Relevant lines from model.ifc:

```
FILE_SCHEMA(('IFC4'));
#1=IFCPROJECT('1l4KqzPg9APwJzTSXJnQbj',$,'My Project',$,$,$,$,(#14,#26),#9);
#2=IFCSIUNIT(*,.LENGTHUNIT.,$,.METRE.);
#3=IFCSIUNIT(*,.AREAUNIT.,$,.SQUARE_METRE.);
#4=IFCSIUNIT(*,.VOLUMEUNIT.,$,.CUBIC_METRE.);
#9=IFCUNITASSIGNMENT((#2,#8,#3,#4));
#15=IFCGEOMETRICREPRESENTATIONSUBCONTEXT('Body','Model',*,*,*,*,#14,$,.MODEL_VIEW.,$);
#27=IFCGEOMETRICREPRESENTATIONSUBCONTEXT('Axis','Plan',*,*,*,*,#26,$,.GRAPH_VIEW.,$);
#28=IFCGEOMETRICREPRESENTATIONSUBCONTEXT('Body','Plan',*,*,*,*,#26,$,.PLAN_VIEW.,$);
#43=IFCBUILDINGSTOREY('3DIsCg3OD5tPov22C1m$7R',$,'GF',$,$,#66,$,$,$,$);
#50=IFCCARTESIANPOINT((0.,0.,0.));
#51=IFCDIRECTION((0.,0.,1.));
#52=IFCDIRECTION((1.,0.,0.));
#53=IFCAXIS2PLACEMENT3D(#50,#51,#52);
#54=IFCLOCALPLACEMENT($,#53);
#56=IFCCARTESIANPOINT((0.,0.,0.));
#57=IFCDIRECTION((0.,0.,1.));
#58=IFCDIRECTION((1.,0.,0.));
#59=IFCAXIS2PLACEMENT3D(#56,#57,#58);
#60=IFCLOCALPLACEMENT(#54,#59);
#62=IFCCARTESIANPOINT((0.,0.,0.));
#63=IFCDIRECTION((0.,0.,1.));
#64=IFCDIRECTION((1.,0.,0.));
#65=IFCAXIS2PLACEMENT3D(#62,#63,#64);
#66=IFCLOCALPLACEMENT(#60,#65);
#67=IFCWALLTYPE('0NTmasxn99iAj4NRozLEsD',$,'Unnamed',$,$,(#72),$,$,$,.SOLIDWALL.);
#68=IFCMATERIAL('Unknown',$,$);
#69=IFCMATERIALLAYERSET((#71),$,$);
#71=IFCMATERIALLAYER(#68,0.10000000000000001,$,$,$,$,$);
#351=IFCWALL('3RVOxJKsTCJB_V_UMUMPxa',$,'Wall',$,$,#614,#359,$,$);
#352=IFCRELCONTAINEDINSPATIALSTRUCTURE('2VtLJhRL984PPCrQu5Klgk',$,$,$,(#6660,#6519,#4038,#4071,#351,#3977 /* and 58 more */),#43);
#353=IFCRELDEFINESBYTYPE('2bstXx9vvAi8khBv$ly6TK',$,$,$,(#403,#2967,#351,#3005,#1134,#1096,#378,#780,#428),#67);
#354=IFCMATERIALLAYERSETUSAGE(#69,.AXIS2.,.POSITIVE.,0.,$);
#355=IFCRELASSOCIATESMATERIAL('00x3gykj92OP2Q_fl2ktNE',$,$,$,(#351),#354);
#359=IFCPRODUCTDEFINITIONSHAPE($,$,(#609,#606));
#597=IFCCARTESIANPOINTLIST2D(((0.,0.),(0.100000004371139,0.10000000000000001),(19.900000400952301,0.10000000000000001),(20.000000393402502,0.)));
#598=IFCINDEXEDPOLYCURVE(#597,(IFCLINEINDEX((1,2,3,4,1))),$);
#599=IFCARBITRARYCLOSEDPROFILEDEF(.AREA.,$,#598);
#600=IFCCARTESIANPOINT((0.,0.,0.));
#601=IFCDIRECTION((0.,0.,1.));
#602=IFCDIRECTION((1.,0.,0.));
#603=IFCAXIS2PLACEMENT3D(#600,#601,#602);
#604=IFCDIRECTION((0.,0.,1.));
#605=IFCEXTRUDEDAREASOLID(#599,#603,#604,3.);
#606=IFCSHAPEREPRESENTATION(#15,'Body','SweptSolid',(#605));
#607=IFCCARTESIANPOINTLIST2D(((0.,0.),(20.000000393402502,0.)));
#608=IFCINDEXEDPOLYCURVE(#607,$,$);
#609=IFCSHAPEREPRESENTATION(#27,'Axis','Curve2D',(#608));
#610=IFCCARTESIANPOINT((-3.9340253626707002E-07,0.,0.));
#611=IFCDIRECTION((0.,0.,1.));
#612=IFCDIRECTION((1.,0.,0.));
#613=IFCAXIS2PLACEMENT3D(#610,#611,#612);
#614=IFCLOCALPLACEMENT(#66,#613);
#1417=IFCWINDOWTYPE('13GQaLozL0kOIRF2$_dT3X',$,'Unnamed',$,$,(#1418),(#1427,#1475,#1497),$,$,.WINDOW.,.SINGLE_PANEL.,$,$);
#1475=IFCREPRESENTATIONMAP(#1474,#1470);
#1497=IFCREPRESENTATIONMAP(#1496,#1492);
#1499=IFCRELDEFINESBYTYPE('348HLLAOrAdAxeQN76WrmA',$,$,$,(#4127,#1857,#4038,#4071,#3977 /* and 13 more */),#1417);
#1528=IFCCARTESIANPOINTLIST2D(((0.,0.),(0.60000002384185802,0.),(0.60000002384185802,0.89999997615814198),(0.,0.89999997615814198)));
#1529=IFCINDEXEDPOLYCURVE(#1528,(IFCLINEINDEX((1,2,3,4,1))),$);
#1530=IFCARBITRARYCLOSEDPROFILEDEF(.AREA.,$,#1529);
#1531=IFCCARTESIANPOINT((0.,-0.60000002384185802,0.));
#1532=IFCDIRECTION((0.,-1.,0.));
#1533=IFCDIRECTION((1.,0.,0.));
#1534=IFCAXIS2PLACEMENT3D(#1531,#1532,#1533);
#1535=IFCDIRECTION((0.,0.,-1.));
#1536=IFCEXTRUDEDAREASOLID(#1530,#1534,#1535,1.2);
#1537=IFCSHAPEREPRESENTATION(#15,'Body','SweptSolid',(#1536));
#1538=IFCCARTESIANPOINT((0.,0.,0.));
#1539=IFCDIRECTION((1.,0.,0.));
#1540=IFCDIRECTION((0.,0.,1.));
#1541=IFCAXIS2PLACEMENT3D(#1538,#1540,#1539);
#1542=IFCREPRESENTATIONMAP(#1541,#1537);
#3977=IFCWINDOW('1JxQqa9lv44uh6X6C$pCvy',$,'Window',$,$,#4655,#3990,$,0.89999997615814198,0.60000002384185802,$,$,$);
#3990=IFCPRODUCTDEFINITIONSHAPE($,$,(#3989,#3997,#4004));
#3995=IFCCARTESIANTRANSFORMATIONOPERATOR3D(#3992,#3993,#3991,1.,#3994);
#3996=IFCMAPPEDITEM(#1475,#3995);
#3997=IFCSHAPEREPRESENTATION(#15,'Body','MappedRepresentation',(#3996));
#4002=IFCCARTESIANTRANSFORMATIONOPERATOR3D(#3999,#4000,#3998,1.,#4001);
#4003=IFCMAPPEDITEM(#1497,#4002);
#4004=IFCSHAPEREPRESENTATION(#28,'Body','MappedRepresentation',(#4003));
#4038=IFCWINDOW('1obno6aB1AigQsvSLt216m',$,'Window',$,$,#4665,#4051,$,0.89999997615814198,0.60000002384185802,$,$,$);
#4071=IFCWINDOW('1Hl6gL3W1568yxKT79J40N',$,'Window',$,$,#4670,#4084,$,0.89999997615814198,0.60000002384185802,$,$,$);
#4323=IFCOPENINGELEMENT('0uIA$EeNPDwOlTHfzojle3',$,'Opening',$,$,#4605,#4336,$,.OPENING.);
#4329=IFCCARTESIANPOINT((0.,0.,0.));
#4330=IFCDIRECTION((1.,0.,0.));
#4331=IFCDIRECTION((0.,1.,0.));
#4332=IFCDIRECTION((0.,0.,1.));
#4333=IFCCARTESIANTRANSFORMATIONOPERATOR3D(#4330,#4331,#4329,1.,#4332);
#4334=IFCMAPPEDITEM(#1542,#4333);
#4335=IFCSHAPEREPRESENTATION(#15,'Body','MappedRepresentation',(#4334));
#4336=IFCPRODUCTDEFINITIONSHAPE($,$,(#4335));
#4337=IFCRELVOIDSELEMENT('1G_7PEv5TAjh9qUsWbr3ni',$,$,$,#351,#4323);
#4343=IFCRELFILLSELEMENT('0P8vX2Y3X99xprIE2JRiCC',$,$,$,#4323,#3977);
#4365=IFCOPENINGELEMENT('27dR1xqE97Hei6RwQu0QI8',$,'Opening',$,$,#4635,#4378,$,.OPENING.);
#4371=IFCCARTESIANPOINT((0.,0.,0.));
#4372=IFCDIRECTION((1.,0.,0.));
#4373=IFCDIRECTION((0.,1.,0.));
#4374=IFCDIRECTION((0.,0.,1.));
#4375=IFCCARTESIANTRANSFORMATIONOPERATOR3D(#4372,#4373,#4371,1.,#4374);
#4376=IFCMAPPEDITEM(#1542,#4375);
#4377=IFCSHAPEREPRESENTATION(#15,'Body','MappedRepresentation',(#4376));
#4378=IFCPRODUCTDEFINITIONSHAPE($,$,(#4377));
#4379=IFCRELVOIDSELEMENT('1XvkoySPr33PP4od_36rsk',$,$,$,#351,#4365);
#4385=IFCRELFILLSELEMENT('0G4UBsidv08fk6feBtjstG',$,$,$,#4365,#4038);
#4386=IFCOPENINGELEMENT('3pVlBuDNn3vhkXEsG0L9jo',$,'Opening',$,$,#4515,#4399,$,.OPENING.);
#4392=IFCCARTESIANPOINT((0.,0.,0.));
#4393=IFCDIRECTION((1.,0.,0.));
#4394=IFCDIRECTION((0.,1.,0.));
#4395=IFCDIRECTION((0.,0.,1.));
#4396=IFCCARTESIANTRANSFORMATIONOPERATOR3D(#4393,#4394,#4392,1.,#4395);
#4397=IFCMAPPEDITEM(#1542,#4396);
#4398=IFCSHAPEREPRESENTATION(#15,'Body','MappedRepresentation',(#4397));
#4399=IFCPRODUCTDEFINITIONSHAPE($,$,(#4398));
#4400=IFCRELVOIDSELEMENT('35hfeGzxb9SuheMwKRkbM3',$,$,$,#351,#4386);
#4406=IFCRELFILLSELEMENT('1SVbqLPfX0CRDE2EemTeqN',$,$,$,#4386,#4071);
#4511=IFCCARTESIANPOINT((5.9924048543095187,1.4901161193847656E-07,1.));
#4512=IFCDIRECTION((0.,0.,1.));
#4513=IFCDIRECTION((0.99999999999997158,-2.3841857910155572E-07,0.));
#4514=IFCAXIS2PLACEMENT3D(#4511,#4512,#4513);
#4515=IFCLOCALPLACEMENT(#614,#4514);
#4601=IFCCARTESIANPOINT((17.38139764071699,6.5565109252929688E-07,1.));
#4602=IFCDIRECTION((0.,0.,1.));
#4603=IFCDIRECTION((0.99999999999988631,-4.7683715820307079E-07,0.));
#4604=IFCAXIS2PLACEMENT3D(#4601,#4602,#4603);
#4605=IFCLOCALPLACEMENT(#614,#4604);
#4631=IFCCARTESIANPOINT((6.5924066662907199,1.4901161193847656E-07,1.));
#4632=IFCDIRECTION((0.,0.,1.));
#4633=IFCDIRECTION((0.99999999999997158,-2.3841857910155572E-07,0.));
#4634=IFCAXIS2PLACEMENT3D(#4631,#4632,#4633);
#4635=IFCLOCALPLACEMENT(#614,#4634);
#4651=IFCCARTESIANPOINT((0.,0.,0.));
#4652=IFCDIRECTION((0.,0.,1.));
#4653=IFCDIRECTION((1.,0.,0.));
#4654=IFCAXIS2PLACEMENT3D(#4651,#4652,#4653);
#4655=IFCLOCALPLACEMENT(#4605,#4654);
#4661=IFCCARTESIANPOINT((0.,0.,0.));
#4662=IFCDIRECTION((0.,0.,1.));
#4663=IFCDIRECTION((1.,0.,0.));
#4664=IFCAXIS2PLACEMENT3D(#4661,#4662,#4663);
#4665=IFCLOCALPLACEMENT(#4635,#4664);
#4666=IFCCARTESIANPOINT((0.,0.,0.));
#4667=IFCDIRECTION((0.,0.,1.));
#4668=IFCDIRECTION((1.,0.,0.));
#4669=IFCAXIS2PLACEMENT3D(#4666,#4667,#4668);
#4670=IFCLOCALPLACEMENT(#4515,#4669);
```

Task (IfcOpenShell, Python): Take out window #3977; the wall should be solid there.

```python
import ifcopenshell
import ifcopenshell.api.feature
import ifcopenshell.api.root
import ifcopenshell.geom
import ifcopenshell.util.shape

model = ifcopenshell.open("model.ifc")
settings = ifcopenshell.geom.settings()


def volume(element):
    """Net volume in cubic metres, openings subtracted."""
    shape = ifcopenshell.geom.create_shape(settings, element)
    return ifcopenshell.util.shape.get_volume(shape.geometry)


window = model.by_guid("1JxQqa9lv44uh6X6C$pCvy")
opening = window.FillsVoids[0].RelatingOpeningElement
wall = opening.VoidsElements[0].RelatingBuildingElement
before = volume(wall)

ifcopenshell.api.root.remove_product(model, product=window)
ifcopenshell.api.feature.remove_feature(model, feature=opening)

after = volume(wall)

print(f"wall volume {before:.3f} -> {after:.3f} m3")

model.write("model_v2.ifc")
```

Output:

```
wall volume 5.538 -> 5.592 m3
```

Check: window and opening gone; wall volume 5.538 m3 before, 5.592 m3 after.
